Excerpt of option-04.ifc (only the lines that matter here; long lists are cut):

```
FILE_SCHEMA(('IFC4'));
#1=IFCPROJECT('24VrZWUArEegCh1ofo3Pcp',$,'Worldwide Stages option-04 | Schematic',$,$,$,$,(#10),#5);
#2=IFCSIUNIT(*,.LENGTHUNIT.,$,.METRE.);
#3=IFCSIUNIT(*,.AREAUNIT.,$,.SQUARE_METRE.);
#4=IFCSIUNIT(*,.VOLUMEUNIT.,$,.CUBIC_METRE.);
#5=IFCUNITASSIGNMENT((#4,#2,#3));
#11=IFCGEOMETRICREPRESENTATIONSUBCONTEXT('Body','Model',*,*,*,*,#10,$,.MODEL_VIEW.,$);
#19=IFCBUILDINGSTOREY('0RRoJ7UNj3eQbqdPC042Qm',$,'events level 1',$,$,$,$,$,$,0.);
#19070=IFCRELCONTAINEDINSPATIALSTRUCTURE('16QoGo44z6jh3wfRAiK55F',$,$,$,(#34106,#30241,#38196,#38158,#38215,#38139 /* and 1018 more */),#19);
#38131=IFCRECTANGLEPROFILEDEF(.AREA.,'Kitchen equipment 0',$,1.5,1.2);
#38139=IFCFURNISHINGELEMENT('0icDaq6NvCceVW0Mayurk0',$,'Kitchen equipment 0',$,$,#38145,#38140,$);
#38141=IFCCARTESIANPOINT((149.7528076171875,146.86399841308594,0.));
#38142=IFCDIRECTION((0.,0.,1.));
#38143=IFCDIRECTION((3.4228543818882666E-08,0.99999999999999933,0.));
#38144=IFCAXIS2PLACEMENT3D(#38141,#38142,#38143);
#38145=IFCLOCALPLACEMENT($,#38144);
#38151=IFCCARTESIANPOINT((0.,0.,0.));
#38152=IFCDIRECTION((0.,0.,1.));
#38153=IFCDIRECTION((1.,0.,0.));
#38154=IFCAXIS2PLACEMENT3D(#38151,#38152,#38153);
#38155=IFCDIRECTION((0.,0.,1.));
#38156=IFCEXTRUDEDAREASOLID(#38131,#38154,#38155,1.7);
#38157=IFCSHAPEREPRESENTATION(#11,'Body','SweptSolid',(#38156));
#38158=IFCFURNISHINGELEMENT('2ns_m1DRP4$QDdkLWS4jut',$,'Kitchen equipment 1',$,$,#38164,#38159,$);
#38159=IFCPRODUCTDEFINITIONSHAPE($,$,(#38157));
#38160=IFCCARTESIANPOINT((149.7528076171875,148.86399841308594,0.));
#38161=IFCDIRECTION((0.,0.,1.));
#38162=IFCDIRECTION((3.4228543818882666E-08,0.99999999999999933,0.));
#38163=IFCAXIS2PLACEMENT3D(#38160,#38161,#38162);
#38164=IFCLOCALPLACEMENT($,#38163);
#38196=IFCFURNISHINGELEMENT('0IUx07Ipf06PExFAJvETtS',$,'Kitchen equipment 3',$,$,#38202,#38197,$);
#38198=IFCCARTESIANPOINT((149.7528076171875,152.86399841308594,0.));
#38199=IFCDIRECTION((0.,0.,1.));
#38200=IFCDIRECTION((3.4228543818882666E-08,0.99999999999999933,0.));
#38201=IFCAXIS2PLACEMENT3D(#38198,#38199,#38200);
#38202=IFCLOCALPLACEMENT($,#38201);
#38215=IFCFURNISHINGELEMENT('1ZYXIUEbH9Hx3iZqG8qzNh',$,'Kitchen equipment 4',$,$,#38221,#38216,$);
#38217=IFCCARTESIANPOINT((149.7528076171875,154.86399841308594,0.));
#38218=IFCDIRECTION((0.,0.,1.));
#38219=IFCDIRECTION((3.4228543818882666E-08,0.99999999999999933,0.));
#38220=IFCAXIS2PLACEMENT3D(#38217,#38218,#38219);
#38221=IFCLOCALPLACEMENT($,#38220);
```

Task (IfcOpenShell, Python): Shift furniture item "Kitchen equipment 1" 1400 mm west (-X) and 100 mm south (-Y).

```python
import ifcopenshell
import ifcopenshell.api.geometry
import ifcopenshell.util.placement
import ifcopenshell.util.unit

model = ifcopenshell.open("option-04.ifc")
unit_scale = ifcopenshell.util.unit.calculate_unit_scale(model)

item = model.by_guid("2ns_m1DRP4$QDdkLWS4jut")
matrix = ifcopenshell.util.placement.get_local_placement(item.ObjectPlacement)
matrix[0, 3] -= 1.4 / unit_scale
matrix[1, 3] -= 0.1 / unit_scale
ifcopenshell.api.geometry.edit_object_placement(model, product=item, matrix=matrix, is_si=False)

print(ifcopenshell.util.placement.get_local_placement(item.ObjectPlacement).round(3) + 0.0)

model.write("option-04-out.ifc")
```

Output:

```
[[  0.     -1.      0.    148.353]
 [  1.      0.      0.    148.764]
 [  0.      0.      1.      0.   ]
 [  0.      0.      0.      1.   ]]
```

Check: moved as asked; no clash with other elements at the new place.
